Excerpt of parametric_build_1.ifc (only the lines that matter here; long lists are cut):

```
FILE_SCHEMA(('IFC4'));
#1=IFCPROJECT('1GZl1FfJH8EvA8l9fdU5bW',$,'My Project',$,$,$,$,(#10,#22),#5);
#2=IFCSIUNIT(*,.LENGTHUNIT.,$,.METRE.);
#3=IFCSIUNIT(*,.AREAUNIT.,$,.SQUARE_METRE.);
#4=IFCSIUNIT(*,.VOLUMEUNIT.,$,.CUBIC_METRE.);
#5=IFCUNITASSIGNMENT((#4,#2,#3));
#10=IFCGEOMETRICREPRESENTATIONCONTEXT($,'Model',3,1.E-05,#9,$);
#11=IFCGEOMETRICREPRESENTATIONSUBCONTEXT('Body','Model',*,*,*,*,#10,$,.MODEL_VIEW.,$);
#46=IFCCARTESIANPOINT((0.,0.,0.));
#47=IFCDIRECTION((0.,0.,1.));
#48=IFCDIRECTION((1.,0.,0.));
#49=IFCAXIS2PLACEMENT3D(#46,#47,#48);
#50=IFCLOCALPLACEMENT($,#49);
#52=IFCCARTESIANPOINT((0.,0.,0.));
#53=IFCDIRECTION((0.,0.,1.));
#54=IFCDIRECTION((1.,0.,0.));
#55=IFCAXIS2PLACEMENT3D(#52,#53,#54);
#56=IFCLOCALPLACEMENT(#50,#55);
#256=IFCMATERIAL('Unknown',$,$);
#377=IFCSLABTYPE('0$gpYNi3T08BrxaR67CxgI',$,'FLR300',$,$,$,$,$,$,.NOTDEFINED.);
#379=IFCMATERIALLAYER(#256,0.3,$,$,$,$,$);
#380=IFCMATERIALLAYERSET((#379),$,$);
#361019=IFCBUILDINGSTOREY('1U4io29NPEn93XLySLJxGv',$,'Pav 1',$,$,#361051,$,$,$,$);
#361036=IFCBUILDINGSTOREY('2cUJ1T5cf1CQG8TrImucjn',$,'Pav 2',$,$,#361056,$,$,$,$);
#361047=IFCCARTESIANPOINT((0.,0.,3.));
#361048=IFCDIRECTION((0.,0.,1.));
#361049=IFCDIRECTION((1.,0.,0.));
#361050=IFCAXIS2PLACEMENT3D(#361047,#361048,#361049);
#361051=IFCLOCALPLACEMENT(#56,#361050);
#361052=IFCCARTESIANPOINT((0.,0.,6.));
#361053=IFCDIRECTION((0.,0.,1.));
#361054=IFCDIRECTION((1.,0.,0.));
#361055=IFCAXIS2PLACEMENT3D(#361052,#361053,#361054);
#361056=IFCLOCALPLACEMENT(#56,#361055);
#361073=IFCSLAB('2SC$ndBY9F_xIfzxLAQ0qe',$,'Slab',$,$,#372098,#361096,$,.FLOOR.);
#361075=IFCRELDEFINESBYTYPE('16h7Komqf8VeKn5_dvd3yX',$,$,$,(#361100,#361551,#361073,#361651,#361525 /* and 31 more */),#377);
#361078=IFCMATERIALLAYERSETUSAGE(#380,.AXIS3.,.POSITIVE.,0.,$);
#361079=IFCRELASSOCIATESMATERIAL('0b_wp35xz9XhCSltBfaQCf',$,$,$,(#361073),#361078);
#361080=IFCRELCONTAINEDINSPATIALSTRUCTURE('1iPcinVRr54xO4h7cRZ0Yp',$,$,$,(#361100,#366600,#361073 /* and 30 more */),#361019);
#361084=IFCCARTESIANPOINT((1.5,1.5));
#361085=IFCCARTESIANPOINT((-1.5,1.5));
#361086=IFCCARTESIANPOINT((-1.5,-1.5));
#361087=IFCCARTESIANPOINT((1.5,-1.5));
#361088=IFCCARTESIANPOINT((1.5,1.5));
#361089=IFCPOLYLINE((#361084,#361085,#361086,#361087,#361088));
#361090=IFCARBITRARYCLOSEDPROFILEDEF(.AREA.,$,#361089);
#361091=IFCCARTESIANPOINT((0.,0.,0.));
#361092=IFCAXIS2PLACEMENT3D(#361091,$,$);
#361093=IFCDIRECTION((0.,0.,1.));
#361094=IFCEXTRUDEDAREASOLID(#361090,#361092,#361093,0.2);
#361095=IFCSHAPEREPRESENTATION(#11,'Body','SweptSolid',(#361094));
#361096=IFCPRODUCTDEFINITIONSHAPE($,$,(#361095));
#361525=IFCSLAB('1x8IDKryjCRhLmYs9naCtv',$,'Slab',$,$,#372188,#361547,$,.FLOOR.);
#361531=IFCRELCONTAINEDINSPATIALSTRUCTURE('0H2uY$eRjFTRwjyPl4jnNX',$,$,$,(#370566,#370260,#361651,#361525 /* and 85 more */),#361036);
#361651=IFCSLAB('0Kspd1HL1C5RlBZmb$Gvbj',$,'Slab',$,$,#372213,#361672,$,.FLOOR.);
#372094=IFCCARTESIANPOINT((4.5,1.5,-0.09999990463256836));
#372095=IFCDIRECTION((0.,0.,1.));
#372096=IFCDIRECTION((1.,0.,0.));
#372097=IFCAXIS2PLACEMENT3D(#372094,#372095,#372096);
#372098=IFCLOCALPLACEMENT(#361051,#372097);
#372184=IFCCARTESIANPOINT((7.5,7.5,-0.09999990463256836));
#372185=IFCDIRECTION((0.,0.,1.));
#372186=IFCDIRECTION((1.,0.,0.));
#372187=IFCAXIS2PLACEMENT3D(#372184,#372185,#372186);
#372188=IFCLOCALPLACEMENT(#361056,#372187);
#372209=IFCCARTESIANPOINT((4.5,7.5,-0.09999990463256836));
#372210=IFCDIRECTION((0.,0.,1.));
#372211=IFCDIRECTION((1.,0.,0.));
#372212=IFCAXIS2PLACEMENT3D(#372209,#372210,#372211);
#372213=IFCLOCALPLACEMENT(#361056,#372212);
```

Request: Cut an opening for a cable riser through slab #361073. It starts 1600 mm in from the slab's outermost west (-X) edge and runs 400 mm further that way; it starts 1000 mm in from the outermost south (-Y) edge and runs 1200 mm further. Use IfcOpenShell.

```python
import numpy as np
import ifcopenshell
import ifcopenshell.api.feature
import ifcopenshell.api.geometry
import ifcopenshell.api.root
import ifcopenshell.geom
import ifcopenshell.util.placement
import ifcopenshell.util.representation
import ifcopenshell.util.shape
import ifcopenshell.util.unit

model = ifcopenshell.open("parametric_build_1.ifc")
unit_scale = ifcopenshell.util.unit.calculate_unit_scale(model)
settings = ifcopenshell.geom.settings()


def volume(element):
    """Net volume in cubic metres, openings subtracted."""
    shape = ifcopenshell.geom.create_shape(settings, element)
    return ifcopenshell.util.shape.get_volume(shape.geometry)


slab = model.by_id(361073)
before = volume(slab)

# Extent in the slab's own axes, in metres. The edges named are its -X and -Y sides.
slab_shape = ifcopenshell.geom.create_shape(settings, slab)
vertices = ifcopenshell.util.shape.get_vertices(slab_shape.geometry)
x_min, y_min, bottom = vertices.min(axis=0)
top = vertices[:, 2].max()

opening = ifcopenshell.api.root.create_entity(model, ifc_class="IfcOpeningElement", name="Cable riser opening", predefined_type="OPENING")
context = ifcopenshell.util.representation.get_context(model, "Model", "Body", "MODEL_VIEW")
width, depth = 0.4, 1.2
outline = [(0.0, 0.0), (width, 0.0), (width, depth), (0.0, depth), (0.0, 0.0)]
# Overshoot both faces by 50 mm so the cut is clean.
shape = ifcopenshell.api.geometry.add_slab_representation(
    model, context=context, depth=top - bottom + 0.1, polyline=outline
)
ifcopenshell.api.geometry.assign_representation(model, product=opening, representation=shape)

matrix = ifcopenshell.util.placement.get_local_placement(slab.ObjectPlacement)
matrix[:, 3] = matrix @ np.append(np.array([x_min + 1.6, y_min + 1, bottom - 0.05]) / unit_scale, 1.0)
ifcopenshell.api.geometry.edit_object_placement(model, product=opening, matrix=matrix, is_si=False)
ifcopenshell.api.feature.add_feature(model, feature=opening, element=slab)

after = volume(slab)

print(f"slab volume {before:.3f} -> {after:.3f} m3")

model.write("parametric_build_1_v2.ifc")
```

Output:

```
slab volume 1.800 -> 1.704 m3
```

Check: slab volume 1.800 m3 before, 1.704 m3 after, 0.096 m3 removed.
